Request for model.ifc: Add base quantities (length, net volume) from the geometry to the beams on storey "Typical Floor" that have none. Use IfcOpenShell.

First a look at what the model holds.

```python
import ifcopenshell
import ifcopenshell.util.element
import ifcopenshell.util.unit

model = ifcopenshell.open("model.ifc")
print(model.schema)
for unit_type in ("LENGTHUNIT", "AREAUNIT", "VOLUMEUNIT"):
    print(unit_type, ifcopenshell.util.unit.calculate_unit_scale(model, unit_type))
storey = next(s for s in model.by_type("IfcBuildingStorey") if s.Name == "Typical Floor")
beams = [e for e in ifcopenshell.util.element.get_decomposition(storey) if e.is_a("IfcBeam")]
for e in sorted(beams, key=lambda e: e.id()):
    print(e.id(), e.is_a(), e.Name, list(ifcopenshell.util.element.get_psets(e, qtos_only=True)), sep=" | ")
```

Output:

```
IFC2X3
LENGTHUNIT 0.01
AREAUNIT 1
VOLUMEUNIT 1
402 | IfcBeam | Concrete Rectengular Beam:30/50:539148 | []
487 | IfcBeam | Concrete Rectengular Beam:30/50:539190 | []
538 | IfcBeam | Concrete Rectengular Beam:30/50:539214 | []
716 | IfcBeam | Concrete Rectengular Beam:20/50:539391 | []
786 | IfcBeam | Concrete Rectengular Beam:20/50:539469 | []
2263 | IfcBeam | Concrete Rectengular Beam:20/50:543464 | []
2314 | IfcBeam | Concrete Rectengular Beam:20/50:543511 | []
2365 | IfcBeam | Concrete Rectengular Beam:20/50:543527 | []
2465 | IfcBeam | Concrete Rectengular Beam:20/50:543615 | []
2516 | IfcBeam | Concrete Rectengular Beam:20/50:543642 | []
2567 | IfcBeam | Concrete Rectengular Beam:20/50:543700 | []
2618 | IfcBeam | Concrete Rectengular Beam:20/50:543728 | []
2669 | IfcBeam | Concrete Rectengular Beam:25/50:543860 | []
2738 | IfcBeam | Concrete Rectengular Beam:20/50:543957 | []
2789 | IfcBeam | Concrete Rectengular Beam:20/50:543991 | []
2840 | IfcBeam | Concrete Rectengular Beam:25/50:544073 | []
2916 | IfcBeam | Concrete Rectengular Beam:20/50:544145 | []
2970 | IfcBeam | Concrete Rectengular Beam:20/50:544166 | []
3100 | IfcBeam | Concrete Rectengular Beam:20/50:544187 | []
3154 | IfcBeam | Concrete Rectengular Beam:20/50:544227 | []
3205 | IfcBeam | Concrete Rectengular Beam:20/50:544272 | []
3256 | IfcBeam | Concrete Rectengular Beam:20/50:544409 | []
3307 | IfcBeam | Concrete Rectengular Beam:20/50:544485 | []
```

```python
import ifcopenshell
import ifcopenshell.api.pset
import ifcopenshell.geom
import ifcopenshell.util.element
import ifcopenshell.util.shape
import ifcopenshell.util.unit

model = ifcopenshell.open("model.ifc")
unit_scale = ifcopenshell.util.unit.calculate_unit_scale(model)
volume_scale = ifcopenshell.util.unit.calculate_unit_scale(model, "VOLUMEUNIT")
settings = ifcopenshell.geom.settings()

storey = next(s for s in model.by_type("IfcBuildingStorey") if s.Name == "Typical Floor")
beams = [e for e in ifcopenshell.util.element.get_decomposition(storey) if e.is_a("IfcBeam")]

for e in sorted(beams, key=lambda e: e.id()):
    if ifcopenshell.util.element.get_psets(e, qtos_only=True, should_inherit=False):
        continue
    # Geometry comes back in metres, in the element's own axes.
    shape = ifcopenshell.geom.create_shape(settings, e)
    values = {
        "Length": ifcopenshell.util.shape.get_max_xyz(shape.geometry) / unit_scale,
        "NetVolume": ifcopenshell.util.shape.get_volume(shape.geometry) / volume_scale,
    }
    qto = ifcopenshell.api.pset.add_qto(model, product=e, name="BaseQuantities")
    ifcopenshell.api.pset.edit_qto(model, qto=qto, properties=values)
    print(e.id(), {k: round(v, 3) for k, v in values.items()})

model.write("model_rev.ifc")
```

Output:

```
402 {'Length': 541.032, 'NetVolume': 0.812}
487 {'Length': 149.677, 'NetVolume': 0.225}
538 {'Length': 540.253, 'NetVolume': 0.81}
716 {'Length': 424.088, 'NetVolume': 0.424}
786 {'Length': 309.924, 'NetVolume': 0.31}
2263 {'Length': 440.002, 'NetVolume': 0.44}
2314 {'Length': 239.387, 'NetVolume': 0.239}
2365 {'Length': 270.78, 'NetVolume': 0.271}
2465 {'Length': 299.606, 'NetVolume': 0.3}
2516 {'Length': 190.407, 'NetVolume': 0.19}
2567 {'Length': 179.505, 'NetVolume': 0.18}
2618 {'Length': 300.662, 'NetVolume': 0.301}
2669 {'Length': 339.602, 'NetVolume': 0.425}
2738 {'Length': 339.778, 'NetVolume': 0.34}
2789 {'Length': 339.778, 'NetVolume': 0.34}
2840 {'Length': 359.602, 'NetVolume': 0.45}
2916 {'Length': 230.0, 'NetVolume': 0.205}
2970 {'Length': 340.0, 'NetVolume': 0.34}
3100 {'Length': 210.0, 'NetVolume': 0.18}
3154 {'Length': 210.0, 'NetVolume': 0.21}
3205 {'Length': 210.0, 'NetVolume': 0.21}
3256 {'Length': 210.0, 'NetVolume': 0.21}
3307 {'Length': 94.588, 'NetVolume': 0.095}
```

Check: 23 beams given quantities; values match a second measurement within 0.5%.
